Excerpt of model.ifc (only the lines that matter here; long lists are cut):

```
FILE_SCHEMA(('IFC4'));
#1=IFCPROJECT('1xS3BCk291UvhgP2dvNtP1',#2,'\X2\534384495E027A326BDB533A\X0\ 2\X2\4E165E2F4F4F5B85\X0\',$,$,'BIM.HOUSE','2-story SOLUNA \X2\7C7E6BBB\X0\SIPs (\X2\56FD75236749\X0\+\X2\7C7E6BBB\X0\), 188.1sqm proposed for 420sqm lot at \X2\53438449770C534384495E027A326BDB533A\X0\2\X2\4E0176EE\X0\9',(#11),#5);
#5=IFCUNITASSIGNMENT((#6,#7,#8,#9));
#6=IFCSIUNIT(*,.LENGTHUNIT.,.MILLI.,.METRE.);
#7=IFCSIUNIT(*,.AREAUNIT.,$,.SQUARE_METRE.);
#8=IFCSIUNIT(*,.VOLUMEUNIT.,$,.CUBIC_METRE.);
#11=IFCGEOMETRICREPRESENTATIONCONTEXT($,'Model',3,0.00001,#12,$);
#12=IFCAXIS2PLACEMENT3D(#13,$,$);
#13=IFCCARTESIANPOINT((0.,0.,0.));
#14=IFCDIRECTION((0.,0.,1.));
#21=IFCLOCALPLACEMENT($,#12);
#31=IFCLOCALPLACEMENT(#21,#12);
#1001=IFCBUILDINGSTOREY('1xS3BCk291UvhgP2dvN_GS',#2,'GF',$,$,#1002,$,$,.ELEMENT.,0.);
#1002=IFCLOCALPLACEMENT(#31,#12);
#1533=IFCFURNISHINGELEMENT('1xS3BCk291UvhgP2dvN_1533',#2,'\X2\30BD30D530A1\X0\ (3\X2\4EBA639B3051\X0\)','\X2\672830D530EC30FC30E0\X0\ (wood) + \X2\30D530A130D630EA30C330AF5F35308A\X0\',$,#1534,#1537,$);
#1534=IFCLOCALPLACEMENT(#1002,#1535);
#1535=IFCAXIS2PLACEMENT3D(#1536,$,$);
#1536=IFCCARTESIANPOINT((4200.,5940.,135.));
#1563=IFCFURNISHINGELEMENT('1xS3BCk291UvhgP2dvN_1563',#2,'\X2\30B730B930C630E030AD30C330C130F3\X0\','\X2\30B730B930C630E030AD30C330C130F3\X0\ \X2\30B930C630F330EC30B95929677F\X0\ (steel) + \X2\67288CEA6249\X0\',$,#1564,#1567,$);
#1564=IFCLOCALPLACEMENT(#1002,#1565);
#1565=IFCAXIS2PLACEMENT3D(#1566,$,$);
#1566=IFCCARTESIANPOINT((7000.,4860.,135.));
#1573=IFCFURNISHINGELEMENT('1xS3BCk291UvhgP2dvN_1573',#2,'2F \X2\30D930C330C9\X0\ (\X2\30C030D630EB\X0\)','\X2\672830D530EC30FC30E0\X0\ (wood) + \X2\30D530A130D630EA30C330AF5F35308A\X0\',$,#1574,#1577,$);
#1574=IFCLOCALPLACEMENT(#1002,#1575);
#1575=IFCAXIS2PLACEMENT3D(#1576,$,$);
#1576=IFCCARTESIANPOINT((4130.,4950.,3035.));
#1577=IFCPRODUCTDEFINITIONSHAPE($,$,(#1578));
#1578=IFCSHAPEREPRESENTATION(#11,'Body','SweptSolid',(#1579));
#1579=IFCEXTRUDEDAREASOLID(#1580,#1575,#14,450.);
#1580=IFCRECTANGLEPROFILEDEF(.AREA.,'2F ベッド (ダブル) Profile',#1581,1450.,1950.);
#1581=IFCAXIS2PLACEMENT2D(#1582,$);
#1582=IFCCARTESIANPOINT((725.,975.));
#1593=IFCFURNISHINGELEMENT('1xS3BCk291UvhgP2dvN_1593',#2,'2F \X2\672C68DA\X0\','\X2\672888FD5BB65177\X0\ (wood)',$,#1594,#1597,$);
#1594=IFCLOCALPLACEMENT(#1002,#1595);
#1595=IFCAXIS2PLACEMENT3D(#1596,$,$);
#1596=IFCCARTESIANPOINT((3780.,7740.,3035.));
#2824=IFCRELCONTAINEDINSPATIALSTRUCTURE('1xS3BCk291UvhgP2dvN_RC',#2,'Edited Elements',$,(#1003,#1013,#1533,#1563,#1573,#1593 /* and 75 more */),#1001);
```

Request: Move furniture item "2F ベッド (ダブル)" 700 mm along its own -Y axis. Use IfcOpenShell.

```python
import ifcopenshell
import ifcopenshell.api.geometry
import ifcopenshell.util.placement
import ifcopenshell.util.unit

model = ifcopenshell.open("model.ifc")
unit_scale = ifcopenshell.util.unit.calculate_unit_scale(model)

item = model.by_guid("1xS3BCk291UvhgP2dvN_1573")
matrix = ifcopenshell.util.placement.get_local_placement(item.ObjectPlacement)
matrix[:3, 3] -= matrix[:3, 1] * 0.7 / unit_scale
ifcopenshell.api.geometry.edit_object_placement(model, product=item, matrix=matrix, is_si=False)

print(ifcopenshell.util.placement.get_local_placement(item.ObjectPlacement).round(3) + 0.0)

model.write("model_updated.ifc")
```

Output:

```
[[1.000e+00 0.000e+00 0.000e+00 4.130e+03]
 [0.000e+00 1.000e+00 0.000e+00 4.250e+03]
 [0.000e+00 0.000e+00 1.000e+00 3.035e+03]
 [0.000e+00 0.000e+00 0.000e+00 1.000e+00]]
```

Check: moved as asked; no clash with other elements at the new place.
